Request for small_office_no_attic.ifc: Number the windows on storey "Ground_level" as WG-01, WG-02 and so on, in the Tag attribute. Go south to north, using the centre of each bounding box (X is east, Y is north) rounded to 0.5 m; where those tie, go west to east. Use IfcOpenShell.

First a look at what the model holds.

```python
import ifcopenshell
import ifcopenshell.util.element
import ifcopenshell.util.placement

model = ifcopenshell.open("small_office_no_attic.ifc")
print(model.schema)
storey = next(s for s in model.by_type("IfcBuildingStorey") if s.Name == "Ground_level")
windows = [e for e in ifcopenshell.util.element.get_decomposition(storey) if e.is_a("IfcWindow")]
for e in sorted(windows, key=lambda e: e.id()):
    origin = ifcopenshell.util.placement.get_local_placement(e.ObjectPlacement)[:3, 3]
    print(e.id(), e.Tag, e.Name, origin.round(2) + 0.0, sep=" | ")
```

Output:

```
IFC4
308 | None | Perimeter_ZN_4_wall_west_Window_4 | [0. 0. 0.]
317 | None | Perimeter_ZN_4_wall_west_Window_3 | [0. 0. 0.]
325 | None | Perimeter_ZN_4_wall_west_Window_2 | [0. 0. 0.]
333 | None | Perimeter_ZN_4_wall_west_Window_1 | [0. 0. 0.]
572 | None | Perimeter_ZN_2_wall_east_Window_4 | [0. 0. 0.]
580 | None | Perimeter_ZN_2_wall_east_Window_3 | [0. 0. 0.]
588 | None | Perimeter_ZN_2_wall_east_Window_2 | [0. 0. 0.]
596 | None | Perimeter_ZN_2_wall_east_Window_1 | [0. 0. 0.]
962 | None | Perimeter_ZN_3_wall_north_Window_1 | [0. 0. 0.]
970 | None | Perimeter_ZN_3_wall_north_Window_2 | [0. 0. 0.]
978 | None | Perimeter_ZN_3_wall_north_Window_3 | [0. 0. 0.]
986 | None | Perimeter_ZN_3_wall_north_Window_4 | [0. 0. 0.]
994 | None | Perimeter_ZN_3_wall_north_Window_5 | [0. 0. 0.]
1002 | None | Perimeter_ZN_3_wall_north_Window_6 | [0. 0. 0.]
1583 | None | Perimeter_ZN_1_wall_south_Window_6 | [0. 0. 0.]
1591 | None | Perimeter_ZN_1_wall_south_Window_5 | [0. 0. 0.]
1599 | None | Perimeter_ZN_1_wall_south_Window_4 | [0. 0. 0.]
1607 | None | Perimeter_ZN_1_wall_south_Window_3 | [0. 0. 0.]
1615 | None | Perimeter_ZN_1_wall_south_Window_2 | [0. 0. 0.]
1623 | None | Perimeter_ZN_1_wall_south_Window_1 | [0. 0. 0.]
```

```python
import ifcopenshell
import ifcopenshell.geom
import ifcopenshell.util.element
import ifcopenshell.util.shape

model = ifcopenshell.open("small_office_no_attic.ifc")
settings = ifcopenshell.geom.settings()
settings.set("use-world-coords", True)


def centre(element):
    shape = ifcopenshell.geom.create_shape(settings, element)
    return ifcopenshell.util.shape.get_bbox_centroid(shape.geometry)


storey = next(s for s in model.by_type("IfcBuildingStorey") if s.Name == "Ground_level")
windows = [e for e in ifcopenshell.util.element.get_decomposition(storey) if e.is_a("IfcWindow")]

# Insertion points can sit at a corner or the storey origin, so sort by the geometry (in metres).
centres = {e: centre(e) for e in windows}
windows.sort(key=lambda e: (round(centres[e][1] / 0.5), centres[e][0]))

for i, e in enumerate(windows, start=1):
    number = f"WG-{i:02d}"
    e.Tag = number
    print(e.id(), number)

model.write("small_office_no_attic-out.ifc")
```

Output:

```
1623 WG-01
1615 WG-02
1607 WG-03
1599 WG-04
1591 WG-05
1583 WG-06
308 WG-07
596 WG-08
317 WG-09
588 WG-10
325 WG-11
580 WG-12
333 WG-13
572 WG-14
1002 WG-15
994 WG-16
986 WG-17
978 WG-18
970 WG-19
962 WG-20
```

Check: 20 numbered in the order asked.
